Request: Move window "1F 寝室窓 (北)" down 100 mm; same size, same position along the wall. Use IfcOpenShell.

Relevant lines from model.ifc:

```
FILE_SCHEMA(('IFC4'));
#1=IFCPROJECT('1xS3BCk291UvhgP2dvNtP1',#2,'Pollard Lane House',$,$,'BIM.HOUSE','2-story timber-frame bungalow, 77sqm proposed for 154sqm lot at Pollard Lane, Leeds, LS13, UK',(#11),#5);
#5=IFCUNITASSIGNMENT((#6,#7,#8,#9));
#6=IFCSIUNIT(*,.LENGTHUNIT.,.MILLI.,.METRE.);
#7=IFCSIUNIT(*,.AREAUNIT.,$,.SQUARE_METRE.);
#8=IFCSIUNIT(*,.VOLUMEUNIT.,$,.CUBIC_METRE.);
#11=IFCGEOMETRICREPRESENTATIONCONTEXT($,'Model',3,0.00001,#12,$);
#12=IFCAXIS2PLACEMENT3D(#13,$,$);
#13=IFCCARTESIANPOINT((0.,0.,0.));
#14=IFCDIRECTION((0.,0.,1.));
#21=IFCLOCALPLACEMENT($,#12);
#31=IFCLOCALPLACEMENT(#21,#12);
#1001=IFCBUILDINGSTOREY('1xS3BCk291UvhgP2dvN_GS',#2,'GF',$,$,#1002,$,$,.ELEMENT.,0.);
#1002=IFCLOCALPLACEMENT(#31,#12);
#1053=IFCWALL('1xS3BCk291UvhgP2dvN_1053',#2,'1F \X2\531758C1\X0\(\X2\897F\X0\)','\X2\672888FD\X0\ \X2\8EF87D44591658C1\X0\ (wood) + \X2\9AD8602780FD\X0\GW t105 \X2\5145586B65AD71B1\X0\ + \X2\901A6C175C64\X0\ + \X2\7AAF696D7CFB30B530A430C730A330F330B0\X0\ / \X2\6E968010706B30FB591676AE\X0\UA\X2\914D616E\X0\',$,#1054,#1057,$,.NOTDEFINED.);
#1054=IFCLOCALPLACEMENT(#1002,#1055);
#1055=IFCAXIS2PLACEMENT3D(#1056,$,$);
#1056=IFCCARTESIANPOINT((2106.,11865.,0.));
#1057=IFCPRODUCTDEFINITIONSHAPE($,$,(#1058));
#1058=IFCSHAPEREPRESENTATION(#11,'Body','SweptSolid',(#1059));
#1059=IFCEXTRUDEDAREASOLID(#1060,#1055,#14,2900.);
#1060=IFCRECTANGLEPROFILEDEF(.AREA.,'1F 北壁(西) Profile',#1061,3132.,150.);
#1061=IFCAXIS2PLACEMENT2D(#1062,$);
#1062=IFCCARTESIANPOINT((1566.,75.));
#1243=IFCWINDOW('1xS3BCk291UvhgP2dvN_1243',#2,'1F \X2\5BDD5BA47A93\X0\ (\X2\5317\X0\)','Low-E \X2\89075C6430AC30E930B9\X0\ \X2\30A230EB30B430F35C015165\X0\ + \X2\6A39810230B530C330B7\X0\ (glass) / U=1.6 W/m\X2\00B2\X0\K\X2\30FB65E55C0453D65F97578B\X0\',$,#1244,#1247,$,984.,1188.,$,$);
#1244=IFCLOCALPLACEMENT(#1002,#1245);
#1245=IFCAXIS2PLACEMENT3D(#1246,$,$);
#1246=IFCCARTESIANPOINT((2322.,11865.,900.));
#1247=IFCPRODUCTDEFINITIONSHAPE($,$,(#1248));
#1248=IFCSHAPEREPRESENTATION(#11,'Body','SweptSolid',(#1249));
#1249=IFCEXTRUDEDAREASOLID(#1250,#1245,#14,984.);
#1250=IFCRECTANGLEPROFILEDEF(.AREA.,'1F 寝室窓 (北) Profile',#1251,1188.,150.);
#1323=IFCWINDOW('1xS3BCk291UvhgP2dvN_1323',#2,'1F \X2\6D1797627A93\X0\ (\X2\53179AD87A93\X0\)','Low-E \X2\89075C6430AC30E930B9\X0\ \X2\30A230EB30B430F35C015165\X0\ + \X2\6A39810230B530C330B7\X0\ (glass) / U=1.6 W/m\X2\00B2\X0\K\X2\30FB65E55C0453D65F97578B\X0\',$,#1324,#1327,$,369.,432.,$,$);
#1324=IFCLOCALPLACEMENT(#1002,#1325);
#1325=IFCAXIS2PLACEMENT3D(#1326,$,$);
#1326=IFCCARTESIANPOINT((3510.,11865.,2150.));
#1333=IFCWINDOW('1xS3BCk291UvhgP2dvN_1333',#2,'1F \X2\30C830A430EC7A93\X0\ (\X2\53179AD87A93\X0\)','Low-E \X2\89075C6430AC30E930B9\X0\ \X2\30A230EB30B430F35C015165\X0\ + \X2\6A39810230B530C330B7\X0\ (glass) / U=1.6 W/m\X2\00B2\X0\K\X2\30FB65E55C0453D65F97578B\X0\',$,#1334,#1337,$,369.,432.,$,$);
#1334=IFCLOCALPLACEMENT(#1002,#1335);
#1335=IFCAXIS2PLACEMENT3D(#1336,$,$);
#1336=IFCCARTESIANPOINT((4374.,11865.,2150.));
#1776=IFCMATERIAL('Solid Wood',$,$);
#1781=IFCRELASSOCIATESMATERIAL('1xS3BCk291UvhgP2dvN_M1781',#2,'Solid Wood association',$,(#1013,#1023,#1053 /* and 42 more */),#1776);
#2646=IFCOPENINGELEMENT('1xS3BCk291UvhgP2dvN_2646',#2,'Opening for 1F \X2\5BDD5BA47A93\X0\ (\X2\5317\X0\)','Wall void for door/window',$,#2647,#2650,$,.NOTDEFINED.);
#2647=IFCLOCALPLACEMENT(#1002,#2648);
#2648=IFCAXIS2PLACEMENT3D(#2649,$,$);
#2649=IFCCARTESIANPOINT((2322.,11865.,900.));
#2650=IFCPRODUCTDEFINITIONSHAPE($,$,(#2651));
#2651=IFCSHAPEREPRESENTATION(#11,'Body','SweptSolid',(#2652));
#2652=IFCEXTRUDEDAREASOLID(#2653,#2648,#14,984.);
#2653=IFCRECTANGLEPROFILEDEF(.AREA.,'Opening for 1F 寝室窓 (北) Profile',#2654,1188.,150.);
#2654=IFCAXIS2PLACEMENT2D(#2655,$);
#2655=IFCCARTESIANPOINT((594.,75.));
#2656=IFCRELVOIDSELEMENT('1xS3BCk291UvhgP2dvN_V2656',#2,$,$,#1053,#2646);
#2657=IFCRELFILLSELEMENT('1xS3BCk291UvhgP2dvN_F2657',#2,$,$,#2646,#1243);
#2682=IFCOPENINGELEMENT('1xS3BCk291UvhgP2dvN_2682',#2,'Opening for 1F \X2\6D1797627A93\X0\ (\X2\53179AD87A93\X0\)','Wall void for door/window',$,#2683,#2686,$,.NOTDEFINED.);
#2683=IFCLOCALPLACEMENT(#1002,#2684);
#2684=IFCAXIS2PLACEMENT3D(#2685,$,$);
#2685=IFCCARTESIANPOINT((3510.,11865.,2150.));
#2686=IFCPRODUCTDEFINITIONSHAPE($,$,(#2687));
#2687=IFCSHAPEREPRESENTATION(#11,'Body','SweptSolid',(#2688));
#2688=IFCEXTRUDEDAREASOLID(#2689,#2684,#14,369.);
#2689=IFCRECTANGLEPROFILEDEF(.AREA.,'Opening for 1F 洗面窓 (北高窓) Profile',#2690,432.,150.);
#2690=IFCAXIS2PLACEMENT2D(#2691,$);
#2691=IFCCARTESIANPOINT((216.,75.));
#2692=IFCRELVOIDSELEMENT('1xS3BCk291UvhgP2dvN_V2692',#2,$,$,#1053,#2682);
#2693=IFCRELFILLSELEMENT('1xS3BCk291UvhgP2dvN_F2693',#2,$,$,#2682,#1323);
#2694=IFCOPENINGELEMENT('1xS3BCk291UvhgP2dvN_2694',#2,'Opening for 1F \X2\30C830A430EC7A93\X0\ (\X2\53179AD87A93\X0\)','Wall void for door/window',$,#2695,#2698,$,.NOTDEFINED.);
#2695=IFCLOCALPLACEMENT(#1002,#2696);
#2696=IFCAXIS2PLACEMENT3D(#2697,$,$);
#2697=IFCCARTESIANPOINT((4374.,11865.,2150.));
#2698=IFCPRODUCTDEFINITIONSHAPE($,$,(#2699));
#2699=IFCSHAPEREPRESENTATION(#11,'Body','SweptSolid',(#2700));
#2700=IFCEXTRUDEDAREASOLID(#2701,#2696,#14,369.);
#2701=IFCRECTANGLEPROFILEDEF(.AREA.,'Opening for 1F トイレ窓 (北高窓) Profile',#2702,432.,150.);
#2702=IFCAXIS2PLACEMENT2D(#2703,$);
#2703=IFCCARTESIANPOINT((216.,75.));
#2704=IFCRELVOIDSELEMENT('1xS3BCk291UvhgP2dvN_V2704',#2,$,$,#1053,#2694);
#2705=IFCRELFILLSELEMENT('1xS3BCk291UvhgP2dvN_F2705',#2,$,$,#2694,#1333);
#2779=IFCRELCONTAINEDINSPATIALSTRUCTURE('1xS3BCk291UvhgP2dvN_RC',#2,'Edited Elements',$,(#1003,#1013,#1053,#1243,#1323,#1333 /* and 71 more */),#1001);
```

```python
import numpy as np
import ifcopenshell
import ifcopenshell.api.geometry
import ifcopenshell.util.placement
import ifcopenshell.util.unit

model = ifcopenshell.open("model.ifc")
unit_scale = ifcopenshell.util.unit.calculate_unit_scale(model)

window = model.by_guid("1xS3BCk291UvhgP2dvN_1243")
opening = window.FillsVoids[0].RelatingOpeningElement
dz = -100.0

shift = np.array([0.0, 0.0, dz])
# The window is not placed relative to its opening, so move both.
for product in (opening, window):
    matrix = ifcopenshell.util.placement.get_local_placement(product.ObjectPlacement)
    matrix[:3, 3] += shift
    ifcopenshell.api.geometry.edit_object_placement(model, product=product, matrix=matrix, is_si=False)

print(f"moved by {dz * unit_scale:+.3f} m")

model.write("model-out.ifc")
```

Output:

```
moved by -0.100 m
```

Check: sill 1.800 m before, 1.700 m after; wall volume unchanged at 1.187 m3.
